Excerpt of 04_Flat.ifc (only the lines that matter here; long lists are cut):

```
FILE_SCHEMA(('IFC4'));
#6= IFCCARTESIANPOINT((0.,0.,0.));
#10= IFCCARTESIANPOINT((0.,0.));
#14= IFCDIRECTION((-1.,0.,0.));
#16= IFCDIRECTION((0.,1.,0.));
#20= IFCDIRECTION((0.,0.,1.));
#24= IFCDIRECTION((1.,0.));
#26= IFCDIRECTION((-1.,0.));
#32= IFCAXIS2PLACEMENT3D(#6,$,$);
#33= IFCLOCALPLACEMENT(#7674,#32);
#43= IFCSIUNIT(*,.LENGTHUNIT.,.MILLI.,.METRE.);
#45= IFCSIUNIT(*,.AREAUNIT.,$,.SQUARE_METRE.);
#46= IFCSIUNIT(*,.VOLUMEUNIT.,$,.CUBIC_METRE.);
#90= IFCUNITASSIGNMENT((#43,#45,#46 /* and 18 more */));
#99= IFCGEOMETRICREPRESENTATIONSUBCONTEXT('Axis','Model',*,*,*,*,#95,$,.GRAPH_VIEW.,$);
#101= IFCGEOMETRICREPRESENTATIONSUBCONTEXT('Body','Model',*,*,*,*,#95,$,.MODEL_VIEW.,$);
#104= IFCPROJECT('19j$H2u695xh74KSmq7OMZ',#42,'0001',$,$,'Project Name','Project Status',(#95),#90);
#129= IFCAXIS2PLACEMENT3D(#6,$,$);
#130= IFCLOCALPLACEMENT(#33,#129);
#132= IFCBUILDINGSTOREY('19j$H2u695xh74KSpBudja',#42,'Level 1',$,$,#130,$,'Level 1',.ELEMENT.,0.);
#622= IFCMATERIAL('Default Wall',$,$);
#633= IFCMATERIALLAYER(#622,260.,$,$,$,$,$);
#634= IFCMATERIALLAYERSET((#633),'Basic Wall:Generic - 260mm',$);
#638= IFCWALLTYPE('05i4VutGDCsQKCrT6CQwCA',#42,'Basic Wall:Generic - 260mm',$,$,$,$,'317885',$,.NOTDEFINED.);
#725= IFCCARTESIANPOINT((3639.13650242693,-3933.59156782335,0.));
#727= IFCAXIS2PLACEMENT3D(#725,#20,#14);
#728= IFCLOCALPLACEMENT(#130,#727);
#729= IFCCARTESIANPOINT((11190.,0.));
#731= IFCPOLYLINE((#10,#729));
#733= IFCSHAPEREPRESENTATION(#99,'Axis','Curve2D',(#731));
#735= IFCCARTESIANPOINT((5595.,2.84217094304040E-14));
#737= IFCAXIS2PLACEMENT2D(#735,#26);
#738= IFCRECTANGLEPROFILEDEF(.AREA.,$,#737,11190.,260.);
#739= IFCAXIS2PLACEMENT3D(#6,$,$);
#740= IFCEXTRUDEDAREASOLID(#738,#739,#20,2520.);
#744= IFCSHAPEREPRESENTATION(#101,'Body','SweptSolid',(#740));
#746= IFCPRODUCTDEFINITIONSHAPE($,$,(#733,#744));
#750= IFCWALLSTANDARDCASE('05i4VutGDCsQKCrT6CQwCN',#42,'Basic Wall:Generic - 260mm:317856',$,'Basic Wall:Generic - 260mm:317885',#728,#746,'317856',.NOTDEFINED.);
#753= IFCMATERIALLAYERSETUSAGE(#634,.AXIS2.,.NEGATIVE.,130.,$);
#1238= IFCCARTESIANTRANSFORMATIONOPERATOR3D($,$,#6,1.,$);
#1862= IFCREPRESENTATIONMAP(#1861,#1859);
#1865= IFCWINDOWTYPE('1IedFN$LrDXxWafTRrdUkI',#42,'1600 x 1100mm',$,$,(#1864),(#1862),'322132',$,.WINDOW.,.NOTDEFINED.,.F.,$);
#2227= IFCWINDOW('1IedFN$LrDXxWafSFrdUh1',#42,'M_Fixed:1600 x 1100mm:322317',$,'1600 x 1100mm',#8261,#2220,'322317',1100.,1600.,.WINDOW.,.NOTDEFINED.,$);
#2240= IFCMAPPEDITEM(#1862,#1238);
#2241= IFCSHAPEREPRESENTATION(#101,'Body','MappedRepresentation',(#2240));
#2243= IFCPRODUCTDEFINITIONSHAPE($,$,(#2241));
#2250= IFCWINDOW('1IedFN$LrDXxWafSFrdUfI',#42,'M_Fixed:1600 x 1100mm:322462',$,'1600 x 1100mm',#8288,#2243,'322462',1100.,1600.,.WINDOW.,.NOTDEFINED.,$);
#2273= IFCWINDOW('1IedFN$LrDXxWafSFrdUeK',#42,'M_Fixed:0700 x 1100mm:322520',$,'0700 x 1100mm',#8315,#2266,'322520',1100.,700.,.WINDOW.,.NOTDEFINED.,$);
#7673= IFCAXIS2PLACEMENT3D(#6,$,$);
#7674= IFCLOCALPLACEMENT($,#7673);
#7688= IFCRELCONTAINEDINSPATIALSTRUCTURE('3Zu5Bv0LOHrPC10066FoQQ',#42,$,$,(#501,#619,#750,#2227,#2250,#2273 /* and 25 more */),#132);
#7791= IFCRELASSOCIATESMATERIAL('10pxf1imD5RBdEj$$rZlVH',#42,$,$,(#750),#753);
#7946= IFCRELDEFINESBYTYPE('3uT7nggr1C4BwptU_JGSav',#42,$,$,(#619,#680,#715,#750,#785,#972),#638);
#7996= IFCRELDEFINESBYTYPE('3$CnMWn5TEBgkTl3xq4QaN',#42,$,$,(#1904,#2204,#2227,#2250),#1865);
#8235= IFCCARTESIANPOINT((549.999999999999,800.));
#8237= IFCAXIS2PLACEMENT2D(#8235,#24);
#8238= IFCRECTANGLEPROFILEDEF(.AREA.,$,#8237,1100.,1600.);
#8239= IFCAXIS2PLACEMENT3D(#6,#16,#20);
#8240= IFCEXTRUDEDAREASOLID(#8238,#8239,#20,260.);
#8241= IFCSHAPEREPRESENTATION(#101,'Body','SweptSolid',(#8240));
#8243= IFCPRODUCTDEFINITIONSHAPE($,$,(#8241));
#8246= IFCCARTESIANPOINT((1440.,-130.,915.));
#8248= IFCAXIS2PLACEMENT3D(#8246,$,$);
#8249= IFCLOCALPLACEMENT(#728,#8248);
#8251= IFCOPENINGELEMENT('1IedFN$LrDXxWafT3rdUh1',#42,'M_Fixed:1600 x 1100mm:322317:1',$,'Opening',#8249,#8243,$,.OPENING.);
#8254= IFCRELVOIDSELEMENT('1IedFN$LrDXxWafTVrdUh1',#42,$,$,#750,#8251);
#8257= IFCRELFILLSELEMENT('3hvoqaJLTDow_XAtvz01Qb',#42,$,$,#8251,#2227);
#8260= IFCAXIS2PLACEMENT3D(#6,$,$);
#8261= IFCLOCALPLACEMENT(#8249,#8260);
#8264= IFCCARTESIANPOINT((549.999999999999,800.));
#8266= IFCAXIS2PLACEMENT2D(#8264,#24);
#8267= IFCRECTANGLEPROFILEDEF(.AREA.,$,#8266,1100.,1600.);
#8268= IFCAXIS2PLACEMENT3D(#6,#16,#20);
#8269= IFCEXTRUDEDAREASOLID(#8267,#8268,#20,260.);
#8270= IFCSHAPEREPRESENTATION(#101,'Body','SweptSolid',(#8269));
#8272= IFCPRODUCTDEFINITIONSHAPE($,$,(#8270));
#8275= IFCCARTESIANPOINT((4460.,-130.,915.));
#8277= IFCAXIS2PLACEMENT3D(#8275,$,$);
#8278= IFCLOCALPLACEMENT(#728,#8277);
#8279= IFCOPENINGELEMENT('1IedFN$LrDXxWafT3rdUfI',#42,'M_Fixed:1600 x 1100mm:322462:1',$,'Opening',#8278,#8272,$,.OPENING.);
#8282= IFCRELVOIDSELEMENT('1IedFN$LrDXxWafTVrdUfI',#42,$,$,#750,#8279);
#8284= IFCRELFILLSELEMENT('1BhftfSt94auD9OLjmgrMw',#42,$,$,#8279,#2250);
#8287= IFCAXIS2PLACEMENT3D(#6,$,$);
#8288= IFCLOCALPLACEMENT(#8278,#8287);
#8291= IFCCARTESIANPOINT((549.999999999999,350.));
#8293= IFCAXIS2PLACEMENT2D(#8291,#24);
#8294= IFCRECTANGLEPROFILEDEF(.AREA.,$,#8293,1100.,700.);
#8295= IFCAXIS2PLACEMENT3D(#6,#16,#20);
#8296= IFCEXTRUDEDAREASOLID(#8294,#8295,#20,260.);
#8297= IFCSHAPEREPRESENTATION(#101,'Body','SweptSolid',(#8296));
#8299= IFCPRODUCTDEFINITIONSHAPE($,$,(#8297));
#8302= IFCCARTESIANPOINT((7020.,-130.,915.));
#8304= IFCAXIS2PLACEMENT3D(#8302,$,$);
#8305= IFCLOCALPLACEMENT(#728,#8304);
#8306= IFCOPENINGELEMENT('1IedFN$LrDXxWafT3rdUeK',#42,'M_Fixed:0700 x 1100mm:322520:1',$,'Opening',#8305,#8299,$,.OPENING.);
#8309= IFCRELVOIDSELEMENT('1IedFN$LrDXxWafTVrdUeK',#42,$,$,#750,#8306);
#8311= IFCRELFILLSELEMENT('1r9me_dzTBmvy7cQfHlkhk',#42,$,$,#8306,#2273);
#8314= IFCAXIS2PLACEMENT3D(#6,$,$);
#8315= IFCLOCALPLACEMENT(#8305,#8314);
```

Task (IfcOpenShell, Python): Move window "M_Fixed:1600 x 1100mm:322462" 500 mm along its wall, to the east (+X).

```python
import ifcopenshell
import ifcopenshell.api.geometry
import ifcopenshell.util.placement
import ifcopenshell.util.unit

model = ifcopenshell.open("04_Flat.ifc")
unit_scale = ifcopenshell.util.unit.calculate_unit_scale(model)

window = model.by_guid("1IedFN$LrDXxWafSFrdUfI")
opening = window.FillsVoids[0].RelatingOpeningElement
wall = opening.VoidsElements[0].RelatingBuildingElement

wall_matrix = ifcopenshell.util.placement.get_local_placement(wall.ObjectPlacement)
shift = wall_matrix[:3, 0] * -0.5 / unit_scale
before = ifcopenshell.util.placement.get_local_placement(window.ObjectPlacement)[:3, 3].copy()

# The window is placed relative to its opening, so it follows when the opening moves.
matrix = ifcopenshell.util.placement.get_local_placement(opening.ObjectPlacement)
matrix[:3, 3] += shift
ifcopenshell.api.geometry.edit_object_placement(
    model, product=opening, matrix=matrix, is_si=False, should_transform_children=True
)

after = ifcopenshell.util.placement.get_local_placement(window.ObjectPlacement)[:3, 3]
print("window moved by", (after - before).round(3) + 0.0)

model.write("04_Flat_v2.ifc")
```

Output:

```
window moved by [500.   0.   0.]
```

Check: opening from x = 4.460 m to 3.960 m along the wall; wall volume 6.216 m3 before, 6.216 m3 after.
